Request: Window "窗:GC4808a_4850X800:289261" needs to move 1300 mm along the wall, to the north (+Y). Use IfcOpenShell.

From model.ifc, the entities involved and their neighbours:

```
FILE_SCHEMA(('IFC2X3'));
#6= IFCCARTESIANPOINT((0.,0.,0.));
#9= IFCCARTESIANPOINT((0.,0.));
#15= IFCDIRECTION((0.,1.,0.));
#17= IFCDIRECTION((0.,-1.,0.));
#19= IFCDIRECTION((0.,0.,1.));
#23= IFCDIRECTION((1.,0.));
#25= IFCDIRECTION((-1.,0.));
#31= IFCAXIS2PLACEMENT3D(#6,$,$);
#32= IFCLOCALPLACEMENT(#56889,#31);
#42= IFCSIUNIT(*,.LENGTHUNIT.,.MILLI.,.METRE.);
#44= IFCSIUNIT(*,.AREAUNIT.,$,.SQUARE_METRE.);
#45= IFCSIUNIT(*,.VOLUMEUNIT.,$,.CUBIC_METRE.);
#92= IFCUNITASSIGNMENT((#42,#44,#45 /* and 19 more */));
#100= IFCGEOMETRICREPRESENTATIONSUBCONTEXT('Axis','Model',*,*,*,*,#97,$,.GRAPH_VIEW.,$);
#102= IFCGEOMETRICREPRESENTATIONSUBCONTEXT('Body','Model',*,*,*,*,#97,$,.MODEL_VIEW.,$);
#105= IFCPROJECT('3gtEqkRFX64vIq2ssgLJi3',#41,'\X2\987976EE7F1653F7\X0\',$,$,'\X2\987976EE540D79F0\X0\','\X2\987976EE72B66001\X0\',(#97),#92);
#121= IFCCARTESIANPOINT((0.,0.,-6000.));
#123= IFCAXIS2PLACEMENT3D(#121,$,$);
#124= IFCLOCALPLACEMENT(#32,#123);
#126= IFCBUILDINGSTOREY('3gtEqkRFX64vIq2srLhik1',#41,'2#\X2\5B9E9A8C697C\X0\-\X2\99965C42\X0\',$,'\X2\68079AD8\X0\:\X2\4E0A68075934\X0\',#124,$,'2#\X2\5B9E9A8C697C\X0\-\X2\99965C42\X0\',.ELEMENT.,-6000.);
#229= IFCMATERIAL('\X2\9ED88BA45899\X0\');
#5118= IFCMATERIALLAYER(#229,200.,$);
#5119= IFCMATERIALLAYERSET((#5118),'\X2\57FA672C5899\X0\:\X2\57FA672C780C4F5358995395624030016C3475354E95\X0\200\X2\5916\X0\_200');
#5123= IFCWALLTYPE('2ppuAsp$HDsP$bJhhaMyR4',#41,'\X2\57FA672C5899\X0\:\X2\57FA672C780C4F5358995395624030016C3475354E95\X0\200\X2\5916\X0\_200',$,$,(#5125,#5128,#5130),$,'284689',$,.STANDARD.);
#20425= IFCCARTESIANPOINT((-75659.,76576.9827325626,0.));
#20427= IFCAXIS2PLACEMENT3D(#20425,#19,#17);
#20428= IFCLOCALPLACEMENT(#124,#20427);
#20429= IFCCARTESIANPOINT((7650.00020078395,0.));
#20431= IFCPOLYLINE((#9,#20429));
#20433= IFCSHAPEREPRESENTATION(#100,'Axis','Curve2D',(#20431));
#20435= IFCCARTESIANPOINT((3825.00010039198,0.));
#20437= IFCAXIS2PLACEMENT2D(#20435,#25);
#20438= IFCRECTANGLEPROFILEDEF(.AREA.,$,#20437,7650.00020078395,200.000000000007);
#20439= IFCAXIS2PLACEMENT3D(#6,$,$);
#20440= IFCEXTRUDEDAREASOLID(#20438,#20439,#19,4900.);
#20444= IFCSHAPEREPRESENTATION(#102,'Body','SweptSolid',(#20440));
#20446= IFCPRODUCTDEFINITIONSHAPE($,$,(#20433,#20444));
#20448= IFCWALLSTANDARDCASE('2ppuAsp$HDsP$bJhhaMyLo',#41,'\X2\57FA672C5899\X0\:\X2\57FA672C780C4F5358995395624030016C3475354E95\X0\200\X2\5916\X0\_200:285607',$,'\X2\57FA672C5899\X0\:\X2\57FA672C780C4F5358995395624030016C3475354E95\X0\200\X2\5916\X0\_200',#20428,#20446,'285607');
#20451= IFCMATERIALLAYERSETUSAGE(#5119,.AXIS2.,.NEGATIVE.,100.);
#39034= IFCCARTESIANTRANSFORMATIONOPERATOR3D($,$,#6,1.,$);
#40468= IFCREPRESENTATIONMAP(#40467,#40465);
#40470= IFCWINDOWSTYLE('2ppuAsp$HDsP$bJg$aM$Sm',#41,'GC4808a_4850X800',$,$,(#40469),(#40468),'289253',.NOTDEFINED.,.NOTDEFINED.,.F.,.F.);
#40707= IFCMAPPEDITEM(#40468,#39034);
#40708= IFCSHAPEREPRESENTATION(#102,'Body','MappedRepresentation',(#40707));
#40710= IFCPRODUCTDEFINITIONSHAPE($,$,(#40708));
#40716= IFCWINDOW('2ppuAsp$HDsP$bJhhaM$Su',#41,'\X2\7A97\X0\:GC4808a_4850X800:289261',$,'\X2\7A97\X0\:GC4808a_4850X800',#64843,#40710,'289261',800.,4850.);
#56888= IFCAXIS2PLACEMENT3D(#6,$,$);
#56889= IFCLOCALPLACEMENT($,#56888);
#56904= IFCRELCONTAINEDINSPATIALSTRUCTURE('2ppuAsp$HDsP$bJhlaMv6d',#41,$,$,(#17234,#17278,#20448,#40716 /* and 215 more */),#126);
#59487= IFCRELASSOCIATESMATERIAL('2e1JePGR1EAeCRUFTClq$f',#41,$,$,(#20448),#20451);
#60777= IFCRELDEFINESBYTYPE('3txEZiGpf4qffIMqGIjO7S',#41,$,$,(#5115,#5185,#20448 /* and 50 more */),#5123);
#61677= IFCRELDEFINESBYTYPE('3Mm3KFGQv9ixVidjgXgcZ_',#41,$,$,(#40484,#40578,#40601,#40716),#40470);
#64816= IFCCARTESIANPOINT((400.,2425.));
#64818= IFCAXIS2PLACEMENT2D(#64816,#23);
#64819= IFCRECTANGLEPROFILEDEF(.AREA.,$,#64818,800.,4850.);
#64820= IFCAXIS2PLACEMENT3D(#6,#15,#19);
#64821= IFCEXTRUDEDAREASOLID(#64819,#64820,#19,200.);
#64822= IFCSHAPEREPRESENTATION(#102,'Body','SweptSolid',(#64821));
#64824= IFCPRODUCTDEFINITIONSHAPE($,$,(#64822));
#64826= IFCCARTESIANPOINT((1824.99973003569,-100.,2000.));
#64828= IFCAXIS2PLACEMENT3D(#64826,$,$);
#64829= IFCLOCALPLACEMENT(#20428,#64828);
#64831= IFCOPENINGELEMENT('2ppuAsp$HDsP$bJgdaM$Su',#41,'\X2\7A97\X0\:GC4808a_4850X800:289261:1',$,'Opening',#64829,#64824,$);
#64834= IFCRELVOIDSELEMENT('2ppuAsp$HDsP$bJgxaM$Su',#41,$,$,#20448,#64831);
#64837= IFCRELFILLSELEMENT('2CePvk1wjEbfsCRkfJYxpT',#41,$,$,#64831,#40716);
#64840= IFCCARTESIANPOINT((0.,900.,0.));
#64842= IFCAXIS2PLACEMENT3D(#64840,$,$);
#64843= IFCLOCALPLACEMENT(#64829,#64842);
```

```python
import ifcopenshell
import ifcopenshell.api.geometry
import ifcopenshell.util.placement
import ifcopenshell.util.unit

model = ifcopenshell.open("model.ifc")
unit_scale = ifcopenshell.util.unit.calculate_unit_scale(model)

window = model.by_guid("2ppuAsp$HDsP$bJhhaM$Su")
opening = window.FillsVoids[0].RelatingOpeningElement
wall = opening.VoidsElements[0].RelatingBuildingElement

wall_matrix = ifcopenshell.util.placement.get_local_placement(wall.ObjectPlacement)
shift = wall_matrix[:3, 0] * -1.3 / unit_scale
before = ifcopenshell.util.placement.get_local_placement(window.ObjectPlacement)[:3, 3].copy()

# The window is placed relative to its opening, so it follows when the opening moves.
matrix = ifcopenshell.util.placement.get_local_placement(opening.ObjectPlacement)
matrix[:3, 3] += shift
ifcopenshell.api.geometry.edit_object_placement(
    model, product=opening, matrix=matrix, is_si=False, should_transform_children=True
)

after = ifcopenshell.util.placement.get_local_placement(window.ObjectPlacement)[:3, 3]
print("window moved by", (after - before).round(3) + 0.0)

model.write("model_v2.ifc")
```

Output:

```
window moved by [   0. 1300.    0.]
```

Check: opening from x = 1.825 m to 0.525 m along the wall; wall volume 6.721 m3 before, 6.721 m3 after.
